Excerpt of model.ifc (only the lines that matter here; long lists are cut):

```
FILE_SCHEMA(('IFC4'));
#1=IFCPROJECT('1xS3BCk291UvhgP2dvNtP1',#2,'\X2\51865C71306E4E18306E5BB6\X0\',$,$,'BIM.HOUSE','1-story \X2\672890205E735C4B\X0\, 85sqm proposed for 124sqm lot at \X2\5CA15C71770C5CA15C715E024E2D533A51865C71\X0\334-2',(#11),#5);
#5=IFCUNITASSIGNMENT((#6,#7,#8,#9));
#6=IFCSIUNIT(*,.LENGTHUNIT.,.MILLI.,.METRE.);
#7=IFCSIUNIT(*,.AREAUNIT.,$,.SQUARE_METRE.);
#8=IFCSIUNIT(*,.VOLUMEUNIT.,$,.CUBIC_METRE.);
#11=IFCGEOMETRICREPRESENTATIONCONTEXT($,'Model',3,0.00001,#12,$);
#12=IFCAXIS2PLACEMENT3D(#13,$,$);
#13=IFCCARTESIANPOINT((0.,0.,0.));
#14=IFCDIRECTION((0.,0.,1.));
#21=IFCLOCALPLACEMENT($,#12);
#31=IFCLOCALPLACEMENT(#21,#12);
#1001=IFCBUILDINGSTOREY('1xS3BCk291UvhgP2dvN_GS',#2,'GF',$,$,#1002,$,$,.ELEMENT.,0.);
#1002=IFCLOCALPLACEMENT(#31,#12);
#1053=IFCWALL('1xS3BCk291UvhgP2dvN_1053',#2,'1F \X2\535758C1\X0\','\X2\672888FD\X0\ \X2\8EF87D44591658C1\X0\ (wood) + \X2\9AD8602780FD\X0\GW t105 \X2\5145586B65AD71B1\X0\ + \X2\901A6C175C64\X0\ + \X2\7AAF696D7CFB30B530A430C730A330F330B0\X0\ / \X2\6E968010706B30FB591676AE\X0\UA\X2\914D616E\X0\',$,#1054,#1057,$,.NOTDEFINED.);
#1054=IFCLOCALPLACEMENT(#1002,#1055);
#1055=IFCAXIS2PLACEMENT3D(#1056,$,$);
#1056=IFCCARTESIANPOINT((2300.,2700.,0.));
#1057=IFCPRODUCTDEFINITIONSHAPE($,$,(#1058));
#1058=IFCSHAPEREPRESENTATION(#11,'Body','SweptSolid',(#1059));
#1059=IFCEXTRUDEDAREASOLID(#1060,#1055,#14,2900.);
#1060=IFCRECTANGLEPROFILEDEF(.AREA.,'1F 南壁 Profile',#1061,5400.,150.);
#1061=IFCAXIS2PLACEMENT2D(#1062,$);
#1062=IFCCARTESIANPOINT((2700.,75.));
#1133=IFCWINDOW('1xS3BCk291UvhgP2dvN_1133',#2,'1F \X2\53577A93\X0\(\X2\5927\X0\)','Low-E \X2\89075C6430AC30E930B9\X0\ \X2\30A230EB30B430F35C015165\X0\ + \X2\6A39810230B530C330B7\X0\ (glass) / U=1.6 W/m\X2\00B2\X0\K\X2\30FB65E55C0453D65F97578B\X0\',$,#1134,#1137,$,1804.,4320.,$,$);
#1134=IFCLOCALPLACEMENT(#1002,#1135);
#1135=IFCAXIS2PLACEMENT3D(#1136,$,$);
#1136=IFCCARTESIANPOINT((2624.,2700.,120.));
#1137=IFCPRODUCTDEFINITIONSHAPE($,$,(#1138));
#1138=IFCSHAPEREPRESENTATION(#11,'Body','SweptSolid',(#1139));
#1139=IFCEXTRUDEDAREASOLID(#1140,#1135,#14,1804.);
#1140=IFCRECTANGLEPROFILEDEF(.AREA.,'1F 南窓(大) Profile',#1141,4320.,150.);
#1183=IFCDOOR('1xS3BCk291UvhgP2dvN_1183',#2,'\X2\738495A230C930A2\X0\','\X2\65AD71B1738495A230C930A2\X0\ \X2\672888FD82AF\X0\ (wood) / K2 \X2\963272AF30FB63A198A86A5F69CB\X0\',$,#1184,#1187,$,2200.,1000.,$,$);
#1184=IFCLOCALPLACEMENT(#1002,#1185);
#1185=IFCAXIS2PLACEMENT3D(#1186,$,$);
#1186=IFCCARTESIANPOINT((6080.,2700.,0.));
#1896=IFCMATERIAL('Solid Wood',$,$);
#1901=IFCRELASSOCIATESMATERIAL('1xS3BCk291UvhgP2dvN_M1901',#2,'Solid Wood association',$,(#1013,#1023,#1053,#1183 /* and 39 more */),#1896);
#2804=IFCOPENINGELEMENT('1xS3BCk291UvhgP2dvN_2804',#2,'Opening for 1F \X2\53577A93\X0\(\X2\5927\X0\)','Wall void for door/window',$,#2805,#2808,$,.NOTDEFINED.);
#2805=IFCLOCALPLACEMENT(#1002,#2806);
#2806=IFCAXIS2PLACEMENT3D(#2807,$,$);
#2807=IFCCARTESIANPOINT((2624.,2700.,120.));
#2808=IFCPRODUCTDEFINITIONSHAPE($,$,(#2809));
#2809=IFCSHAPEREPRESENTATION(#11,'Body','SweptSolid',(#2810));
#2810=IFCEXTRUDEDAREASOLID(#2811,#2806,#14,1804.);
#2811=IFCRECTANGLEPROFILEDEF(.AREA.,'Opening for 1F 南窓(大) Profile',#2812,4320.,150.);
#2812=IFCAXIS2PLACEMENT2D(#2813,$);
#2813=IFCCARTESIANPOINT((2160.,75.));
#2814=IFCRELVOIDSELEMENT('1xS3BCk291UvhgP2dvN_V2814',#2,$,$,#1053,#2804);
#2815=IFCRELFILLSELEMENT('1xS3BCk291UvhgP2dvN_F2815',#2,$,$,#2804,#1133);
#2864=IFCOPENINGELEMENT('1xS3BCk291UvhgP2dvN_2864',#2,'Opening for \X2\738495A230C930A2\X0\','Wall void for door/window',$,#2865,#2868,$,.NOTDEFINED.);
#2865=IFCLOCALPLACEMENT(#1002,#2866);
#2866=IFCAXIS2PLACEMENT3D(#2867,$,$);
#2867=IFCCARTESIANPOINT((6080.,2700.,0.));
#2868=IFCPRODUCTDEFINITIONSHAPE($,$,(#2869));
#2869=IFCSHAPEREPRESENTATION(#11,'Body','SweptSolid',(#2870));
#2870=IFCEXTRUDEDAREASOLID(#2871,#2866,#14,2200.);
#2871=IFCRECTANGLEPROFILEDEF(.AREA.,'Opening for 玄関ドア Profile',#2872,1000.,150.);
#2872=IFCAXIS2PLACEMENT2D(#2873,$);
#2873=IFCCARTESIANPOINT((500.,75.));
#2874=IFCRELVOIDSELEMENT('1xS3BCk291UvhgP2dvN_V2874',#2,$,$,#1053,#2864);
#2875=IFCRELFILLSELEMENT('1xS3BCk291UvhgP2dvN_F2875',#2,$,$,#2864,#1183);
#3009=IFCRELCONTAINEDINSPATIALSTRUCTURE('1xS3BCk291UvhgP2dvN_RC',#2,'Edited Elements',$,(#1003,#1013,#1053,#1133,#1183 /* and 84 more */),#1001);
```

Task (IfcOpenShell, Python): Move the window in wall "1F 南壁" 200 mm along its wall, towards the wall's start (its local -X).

```python
import ifcopenshell
import ifcopenshell.api.geometry
import ifcopenshell.util.placement

model = ifcopenshell.open("model.ifc")

window = model.by_id(1133)
opening = window.FillsVoids[0].RelatingOpeningElement
wall = opening.VoidsElements[0].RelatingBuildingElement

wall_matrix = ifcopenshell.util.placement.get_local_placement(wall.ObjectPlacement)
shift = wall_matrix[:3, 0] * -200.0
before = ifcopenshell.util.placement.get_local_placement(window.ObjectPlacement)[:3, 3].copy()

# The window is not placed relative to its opening, so move both.
for product in (opening, window):
    matrix = ifcopenshell.util.placement.get_local_placement(product.ObjectPlacement)
    matrix[:3, 3] += shift
    ifcopenshell.api.geometry.edit_object_placement(model, product=product, matrix=matrix, is_si=False)

after = ifcopenshell.util.placement.get_local_placement(window.ObjectPlacement)[:3, 3]
print("window moved by", (after - before).round(3) + 0.0)

model.write("model_rev.ifc")
```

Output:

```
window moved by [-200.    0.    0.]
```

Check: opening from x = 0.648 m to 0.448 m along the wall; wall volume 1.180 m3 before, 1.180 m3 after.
